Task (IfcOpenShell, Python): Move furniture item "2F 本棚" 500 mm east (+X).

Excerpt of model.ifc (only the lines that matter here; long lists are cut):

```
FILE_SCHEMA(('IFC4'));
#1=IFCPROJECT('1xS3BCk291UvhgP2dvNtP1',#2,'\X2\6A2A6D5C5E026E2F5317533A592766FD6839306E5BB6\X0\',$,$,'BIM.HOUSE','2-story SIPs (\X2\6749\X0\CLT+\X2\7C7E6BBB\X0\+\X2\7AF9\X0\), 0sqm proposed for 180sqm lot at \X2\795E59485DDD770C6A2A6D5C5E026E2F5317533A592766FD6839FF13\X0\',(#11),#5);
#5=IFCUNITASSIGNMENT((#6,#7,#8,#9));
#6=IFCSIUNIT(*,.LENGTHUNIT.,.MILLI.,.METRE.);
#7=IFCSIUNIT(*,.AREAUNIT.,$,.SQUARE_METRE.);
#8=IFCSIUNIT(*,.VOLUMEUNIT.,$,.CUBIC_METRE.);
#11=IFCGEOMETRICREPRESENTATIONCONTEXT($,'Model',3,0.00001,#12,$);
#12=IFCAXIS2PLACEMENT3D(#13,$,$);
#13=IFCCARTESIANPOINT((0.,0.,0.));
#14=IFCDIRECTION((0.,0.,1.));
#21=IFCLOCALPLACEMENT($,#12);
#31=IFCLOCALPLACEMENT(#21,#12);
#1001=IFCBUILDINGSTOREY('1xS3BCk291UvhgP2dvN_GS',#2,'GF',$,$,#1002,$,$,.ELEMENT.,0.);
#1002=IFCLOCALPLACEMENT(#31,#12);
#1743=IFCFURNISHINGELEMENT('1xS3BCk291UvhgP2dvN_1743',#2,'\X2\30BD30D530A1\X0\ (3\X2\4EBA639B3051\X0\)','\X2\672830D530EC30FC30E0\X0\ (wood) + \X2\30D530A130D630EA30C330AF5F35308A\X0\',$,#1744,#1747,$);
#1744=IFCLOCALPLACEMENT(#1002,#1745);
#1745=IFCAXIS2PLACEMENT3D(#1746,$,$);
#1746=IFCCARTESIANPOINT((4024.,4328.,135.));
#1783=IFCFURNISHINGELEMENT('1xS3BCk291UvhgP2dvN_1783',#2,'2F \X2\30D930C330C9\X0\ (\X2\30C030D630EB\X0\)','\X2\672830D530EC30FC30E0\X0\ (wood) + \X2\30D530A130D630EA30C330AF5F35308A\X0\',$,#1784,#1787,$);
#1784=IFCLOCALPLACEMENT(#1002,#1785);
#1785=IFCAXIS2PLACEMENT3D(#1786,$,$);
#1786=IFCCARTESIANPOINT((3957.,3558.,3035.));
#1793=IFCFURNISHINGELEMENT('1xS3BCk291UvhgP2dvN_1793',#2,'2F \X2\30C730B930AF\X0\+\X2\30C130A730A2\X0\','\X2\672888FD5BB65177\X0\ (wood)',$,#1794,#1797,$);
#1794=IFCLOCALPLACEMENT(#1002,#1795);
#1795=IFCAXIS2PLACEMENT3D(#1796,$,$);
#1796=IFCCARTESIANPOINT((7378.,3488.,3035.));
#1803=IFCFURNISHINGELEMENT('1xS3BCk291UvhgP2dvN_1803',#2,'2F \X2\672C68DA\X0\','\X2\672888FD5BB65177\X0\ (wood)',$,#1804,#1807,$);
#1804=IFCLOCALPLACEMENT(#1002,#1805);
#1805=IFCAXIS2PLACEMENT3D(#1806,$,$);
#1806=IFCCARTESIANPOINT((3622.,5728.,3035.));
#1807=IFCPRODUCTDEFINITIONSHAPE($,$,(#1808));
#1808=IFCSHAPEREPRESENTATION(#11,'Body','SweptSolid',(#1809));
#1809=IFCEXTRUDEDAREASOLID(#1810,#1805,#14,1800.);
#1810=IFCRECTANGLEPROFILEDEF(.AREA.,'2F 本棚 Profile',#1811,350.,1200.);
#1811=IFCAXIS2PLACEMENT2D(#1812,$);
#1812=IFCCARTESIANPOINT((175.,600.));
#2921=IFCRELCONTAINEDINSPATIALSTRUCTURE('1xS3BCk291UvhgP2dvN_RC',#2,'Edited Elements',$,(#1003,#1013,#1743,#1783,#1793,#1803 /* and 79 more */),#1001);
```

```python
import ifcopenshell
import ifcopenshell.api.geometry
import ifcopenshell.util.placement

model = ifcopenshell.open("model.ifc")

item = model.by_guid("1xS3BCk291UvhgP2dvN_1803")
matrix = ifcopenshell.util.placement.get_local_placement(item.ObjectPlacement)
matrix[0, 3] += 500.0
ifcopenshell.api.geometry.edit_object_placement(model, product=item, matrix=matrix, is_si=False)

print(ifcopenshell.util.placement.get_local_placement(item.ObjectPlacement).round(3) + 0.0)

model.write("model_v2.ifc")
```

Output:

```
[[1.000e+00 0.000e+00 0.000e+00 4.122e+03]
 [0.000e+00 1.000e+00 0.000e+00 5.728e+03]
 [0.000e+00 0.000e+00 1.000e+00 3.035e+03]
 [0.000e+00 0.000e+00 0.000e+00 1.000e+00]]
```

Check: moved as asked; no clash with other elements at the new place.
